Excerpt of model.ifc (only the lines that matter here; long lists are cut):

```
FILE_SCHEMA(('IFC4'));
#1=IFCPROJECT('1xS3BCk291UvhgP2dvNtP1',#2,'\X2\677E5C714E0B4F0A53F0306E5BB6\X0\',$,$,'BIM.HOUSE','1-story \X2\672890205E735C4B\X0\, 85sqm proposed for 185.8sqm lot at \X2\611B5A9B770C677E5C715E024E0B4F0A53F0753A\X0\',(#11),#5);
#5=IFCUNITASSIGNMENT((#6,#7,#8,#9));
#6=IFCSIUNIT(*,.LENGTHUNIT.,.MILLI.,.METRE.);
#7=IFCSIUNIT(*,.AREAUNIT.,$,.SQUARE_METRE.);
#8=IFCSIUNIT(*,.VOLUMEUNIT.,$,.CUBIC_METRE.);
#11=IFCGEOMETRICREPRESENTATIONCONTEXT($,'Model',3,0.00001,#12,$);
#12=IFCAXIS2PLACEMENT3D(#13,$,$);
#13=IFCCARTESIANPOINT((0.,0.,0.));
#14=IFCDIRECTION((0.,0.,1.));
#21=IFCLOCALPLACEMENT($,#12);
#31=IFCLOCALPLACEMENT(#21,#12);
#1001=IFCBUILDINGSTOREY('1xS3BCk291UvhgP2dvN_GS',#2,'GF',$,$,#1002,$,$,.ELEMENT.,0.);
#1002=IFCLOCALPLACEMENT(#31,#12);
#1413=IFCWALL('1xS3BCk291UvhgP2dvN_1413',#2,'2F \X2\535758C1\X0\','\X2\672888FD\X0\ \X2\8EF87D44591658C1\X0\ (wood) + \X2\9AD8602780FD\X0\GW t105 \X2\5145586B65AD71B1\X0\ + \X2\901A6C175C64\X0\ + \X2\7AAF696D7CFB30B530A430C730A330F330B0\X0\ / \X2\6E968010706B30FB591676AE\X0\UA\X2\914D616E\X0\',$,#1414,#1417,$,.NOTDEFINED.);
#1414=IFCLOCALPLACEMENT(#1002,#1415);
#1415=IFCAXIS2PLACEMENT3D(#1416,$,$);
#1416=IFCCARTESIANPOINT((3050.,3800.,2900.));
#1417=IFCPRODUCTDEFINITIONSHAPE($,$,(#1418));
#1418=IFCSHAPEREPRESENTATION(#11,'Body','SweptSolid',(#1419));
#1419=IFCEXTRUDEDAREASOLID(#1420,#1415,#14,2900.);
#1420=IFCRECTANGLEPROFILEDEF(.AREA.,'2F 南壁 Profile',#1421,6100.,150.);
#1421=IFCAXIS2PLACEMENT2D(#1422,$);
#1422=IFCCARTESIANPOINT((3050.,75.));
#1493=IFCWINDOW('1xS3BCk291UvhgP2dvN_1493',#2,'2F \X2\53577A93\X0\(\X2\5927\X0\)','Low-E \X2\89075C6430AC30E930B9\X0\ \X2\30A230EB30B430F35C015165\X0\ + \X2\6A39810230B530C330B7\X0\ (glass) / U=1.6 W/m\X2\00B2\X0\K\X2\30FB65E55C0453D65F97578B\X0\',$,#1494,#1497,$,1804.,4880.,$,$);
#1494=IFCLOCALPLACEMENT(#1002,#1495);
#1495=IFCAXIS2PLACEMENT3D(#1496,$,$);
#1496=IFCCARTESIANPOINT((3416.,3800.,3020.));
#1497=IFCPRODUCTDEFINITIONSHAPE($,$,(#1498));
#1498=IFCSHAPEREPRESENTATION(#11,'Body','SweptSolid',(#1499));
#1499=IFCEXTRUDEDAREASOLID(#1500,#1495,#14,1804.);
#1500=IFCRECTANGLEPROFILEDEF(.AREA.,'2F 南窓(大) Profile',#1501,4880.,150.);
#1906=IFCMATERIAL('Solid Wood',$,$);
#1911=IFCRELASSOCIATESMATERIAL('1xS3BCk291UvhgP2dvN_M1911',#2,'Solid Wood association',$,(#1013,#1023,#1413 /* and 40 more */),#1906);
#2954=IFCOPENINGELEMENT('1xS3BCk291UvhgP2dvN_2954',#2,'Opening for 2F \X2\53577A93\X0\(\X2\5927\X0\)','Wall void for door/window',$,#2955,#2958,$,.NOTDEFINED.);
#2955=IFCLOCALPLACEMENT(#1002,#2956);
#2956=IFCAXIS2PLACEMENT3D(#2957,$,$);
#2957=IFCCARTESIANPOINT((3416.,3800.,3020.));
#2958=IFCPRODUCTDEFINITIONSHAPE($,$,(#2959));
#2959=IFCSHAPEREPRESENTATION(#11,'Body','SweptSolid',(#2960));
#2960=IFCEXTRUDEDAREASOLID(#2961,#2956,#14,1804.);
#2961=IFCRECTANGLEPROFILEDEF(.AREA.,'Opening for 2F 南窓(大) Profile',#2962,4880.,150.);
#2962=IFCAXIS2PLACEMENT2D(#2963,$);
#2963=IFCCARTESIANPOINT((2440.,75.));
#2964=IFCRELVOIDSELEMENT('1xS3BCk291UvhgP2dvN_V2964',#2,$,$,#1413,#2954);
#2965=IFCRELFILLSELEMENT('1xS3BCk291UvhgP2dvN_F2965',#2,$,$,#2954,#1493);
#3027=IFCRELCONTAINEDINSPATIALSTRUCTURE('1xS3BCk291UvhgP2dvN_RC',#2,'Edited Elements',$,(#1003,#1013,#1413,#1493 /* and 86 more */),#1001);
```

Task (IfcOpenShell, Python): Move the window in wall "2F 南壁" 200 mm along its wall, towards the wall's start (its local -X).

```python
import ifcopenshell
import ifcopenshell.api.geometry
import ifcopenshell.util.placement
import ifcopenshell.util.unit

model = ifcopenshell.open("model.ifc")
unit_scale = ifcopenshell.util.unit.calculate_unit_scale(model)

window = model.by_guid("1xS3BCk291UvhgP2dvN_1493")
opening = window.FillsVoids[0].RelatingOpeningElement
wall = opening.VoidsElements[0].RelatingBuildingElement

wall_matrix = ifcopenshell.util.placement.get_local_placement(wall.ObjectPlacement)
shift = wall_matrix[:3, 0] * -0.2 / unit_scale
before = ifcopenshell.util.placement.get_local_placement(window.ObjectPlacement)[:3, 3].copy()

# The window is not placed relative to its opening, so move both.
for product in (opening, window):
    matrix = ifcopenshell.util.placement.get_local_placement(product.ObjectPlacement)
    matrix[:3, 3] += shift
    ifcopenshell.api.geometry.edit_object_placement(model, product=product, matrix=matrix, is_si=False)

after = ifcopenshell.util.placement.get_local_placement(window.ObjectPlacement)[:3, 3]
print("window moved by", (after - before).round(3) + 0.0)

model.write("model_updated.ifc")
```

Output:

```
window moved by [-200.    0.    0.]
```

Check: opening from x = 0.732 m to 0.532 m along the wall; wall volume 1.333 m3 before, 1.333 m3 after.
